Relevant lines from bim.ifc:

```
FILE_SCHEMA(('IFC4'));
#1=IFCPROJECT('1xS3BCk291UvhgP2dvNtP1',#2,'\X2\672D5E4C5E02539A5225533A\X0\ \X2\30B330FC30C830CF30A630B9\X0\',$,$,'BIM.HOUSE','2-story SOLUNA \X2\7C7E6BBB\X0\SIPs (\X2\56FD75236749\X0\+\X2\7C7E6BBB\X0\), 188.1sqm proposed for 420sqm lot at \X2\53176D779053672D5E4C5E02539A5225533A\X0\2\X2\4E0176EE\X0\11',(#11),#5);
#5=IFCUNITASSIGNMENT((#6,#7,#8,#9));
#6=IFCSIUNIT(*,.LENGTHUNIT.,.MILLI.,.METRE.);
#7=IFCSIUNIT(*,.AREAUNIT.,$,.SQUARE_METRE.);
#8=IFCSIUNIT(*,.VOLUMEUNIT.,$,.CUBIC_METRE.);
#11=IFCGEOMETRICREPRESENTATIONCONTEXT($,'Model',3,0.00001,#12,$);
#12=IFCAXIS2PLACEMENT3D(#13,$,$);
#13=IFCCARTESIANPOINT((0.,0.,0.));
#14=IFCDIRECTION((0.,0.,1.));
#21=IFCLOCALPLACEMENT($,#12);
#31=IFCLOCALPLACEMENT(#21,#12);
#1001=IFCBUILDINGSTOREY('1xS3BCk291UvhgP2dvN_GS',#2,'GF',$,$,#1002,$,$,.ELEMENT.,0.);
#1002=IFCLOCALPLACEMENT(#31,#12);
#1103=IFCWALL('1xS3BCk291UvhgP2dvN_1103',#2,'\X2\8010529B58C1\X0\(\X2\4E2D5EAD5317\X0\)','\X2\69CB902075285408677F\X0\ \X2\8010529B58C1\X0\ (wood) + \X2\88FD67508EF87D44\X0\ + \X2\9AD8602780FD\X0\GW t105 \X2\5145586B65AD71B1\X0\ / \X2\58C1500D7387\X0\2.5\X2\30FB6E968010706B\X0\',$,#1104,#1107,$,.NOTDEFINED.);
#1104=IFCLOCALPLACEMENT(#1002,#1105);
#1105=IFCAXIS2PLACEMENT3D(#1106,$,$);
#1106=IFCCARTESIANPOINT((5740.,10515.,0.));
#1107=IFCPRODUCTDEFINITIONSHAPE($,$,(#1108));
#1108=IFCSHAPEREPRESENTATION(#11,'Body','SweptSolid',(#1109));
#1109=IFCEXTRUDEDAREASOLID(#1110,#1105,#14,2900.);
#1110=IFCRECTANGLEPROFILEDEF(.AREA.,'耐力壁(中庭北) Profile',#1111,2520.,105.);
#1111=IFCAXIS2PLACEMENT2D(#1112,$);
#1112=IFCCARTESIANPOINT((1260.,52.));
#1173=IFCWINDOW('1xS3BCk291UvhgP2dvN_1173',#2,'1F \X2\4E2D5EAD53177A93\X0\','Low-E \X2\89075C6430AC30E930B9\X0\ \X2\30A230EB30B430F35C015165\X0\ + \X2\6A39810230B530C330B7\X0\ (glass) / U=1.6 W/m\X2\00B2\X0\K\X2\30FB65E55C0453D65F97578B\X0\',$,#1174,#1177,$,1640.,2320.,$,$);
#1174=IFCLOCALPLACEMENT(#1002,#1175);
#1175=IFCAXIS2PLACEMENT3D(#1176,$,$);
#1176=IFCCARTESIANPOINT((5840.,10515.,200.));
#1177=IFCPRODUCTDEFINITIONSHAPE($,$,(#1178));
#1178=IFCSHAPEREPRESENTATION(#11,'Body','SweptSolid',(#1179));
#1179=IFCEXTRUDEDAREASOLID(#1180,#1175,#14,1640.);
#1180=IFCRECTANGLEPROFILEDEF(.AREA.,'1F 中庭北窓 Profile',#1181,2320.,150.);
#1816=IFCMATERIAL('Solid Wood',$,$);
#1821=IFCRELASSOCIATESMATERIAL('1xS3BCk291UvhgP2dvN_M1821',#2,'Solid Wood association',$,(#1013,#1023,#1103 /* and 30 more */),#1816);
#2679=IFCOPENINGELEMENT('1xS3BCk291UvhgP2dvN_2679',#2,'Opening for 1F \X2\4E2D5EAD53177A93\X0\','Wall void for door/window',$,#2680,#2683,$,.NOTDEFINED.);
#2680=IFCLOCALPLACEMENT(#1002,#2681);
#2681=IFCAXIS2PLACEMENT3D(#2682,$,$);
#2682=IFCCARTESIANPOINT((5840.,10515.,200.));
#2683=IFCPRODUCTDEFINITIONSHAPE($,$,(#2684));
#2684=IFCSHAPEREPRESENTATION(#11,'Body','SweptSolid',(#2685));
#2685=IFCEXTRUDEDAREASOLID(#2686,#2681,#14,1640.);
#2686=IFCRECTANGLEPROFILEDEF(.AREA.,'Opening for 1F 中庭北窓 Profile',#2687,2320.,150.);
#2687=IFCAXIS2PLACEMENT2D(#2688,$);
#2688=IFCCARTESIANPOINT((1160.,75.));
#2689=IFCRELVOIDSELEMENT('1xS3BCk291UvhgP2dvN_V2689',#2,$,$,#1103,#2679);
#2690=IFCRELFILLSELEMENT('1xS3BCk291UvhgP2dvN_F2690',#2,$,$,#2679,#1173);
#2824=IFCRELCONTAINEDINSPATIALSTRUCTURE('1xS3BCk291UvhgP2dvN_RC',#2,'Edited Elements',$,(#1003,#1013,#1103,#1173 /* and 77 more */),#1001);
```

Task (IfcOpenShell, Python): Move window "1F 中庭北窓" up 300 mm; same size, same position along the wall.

```python
import numpy as np
import ifcopenshell
import ifcopenshell.api.geometry
import ifcopenshell.util.placement
import ifcopenshell.util.unit

model = ifcopenshell.open("bim.ifc")
unit_scale = ifcopenshell.util.unit.calculate_unit_scale(model)

window = model.by_id(1173)
opening = window.FillsVoids[0].RelatingOpeningElement
dz = 0.3 / unit_scale

shift = np.array([0.0, 0.0, dz])
# The window is not placed relative to its opening, so move both.
for product in (opening, window):
    matrix = ifcopenshell.util.placement.get_local_placement(product.ObjectPlacement)
    matrix[:3, 3] += shift
    ifcopenshell.api.geometry.edit_object_placement(model, product=product, matrix=matrix, is_si=False)

print(f"moved by {dz * unit_scale:+.3f} m")

model.write("bim_v2.ifc")
```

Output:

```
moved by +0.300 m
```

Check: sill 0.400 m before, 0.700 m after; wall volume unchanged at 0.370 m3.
